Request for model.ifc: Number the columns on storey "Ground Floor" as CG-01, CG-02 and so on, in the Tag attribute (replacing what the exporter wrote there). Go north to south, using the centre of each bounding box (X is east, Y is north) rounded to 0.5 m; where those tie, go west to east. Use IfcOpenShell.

First a look at what the model holds.

```python
import ifcopenshell
import ifcopenshell.util.element
import ifcopenshell.util.placement

model = ifcopenshell.open("model.ifc")
print(model.schema)
storey = next(s for s in model.by_type("IfcBuildingStorey") if s.Name == "Ground Floor")
columns = [e for e in ifcopenshell.util.element.get_decomposition(storey) if e.is_a("IfcColumn")]
for e in sorted(columns, key=lambda e: e.id()):
    origin = ifcopenshell.util.placement.get_local_placement(e.ObjectPlacement)[:3, 3]
    print(e.id(), e.Tag, e.Name, origin.round(2) + 0.0, sep=" | ")
```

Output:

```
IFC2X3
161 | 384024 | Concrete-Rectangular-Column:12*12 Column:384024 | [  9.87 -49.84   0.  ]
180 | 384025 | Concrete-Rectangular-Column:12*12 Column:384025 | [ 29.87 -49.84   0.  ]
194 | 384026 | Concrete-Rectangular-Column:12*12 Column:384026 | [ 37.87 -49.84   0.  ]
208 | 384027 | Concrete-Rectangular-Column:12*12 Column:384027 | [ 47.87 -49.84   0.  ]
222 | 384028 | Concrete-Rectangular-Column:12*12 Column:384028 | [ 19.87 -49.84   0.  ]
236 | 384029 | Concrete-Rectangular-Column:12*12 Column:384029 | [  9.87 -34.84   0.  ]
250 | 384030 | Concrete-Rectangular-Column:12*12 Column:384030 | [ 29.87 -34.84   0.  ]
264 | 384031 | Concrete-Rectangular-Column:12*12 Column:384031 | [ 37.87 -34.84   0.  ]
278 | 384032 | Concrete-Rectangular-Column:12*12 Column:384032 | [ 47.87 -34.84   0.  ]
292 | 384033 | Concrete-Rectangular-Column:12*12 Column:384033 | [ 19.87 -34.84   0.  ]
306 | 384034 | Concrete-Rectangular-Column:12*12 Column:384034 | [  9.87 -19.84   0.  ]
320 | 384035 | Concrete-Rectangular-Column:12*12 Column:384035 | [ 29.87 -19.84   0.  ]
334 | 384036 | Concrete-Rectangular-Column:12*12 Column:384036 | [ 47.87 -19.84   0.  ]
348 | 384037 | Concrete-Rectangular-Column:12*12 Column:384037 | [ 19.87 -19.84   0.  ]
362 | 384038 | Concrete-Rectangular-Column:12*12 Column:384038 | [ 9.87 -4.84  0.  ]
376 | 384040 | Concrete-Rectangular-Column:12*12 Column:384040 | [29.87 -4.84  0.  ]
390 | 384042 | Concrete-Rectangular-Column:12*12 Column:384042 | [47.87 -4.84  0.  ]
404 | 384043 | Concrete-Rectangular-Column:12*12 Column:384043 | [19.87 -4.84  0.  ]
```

```python
import ifcopenshell
import ifcopenshell.geom
import ifcopenshell.util.element
import ifcopenshell.util.shape

model = ifcopenshell.open("model.ifc")
settings = ifcopenshell.geom.settings()
settings.set("use-world-coords", True)


def centre(element):
    shape = ifcopenshell.geom.create_shape(settings, element)
    return ifcopenshell.util.shape.get_bbox_centroid(shape.geometry)


storey = next(s for s in model.by_type("IfcBuildingStorey") if s.Name == "Ground Floor")
columns = [e for e in ifcopenshell.util.element.get_decomposition(storey) if e.is_a("IfcColumn")]

# Insertion points can sit at a corner or the storey origin, so sort by the geometry (in metres).
centres = {e: centre(e) for e in columns}
columns.sort(key=lambda e: (-round(centres[e][1] / 0.5), centres[e][0]))

for i, e in enumerate(columns, start=1):
    number = f"CG-{i:02d}"
    e.Tag = number
    print(e.id(), number)

model.write("model-out.ifc")
```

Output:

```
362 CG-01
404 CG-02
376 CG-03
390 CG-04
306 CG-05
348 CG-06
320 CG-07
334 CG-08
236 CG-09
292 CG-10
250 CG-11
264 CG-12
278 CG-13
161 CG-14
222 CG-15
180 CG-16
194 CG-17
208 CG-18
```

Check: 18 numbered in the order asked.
